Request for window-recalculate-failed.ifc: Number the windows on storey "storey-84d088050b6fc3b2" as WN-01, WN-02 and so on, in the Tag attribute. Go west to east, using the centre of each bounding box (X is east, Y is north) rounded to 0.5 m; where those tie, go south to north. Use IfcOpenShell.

First a look at what the model holds.

```python
import ifcopenshell
import ifcopenshell.util.element
import ifcopenshell.util.placement

model = ifcopenshell.open("window-recalculate-failed.ifc")
print(model.schema)
storey = next(s for s in model.by_type("IfcBuildingStorey") if s.Name == "storey-84d088050b6fc3b2")
windows = [e for e in ifcopenshell.util.element.get_decomposition(storey) if e.is_a("IfcWindow")]
for e in sorted(windows, key=lambda e: e.id()):
    origin = ifcopenshell.util.placement.get_local_placement(e.ObjectPlacement)[:3, 3]
    print(e.id(), e.Tag, e.Name, origin.round(2) + 0.0, sep=" | ")
```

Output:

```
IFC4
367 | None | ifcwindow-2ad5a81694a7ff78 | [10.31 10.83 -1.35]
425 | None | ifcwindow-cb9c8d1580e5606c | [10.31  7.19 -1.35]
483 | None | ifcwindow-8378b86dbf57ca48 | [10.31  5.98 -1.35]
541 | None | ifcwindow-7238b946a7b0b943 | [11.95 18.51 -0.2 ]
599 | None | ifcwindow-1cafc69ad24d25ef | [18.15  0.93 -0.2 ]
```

```python
import ifcopenshell
import ifcopenshell.geom
import ifcopenshell.util.element
import ifcopenshell.util.shape

model = ifcopenshell.open("window-recalculate-failed.ifc")
settings = ifcopenshell.geom.settings()
settings.set("use-world-coords", True)


def centre(element):
    shape = ifcopenshell.geom.create_shape(settings, element)
    return ifcopenshell.util.shape.get_bbox_centroid(shape.geometry)


storey = next(s for s in model.by_type("IfcBuildingStorey") if s.Name == "storey-84d088050b6fc3b2")
windows = [e for e in ifcopenshell.util.element.get_decomposition(storey) if e.is_a("IfcWindow")]

# Insertion points can sit at a corner or the storey origin, so sort by the geometry (in metres).
centres = {e: centre(e) for e in windows}
windows.sort(key=lambda e: (round(centres[e][0] / 0.5), centres[e][1]))

for i, e in enumerate(windows, start=1):
    number = f"WN-{i:02d}"
    e.Tag = number
    print(e.id(), number)

model.write("window-recalculate-failed_edited.ifc")
```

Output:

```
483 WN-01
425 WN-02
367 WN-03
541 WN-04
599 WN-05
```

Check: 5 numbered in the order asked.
